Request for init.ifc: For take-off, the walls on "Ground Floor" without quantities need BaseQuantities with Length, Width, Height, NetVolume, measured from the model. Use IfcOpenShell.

First a look at what the model holds.

```python
import ifcopenshell
import ifcopenshell.util.element
import ifcopenshell.util.unit

model = ifcopenshell.open("init.ifc")
print(model.schema)
for unit_type in ("LENGTHUNIT", "AREAUNIT", "VOLUMEUNIT"):
    print(unit_type, ifcopenshell.util.unit.calculate_unit_scale(model, unit_type))
storey = next(s for s in model.by_type("IfcBuildingStorey") if s.Name == "Ground Floor")
walls = [e for e in ifcopenshell.util.element.get_decomposition(storey) if e.is_a("IfcWall")]
for e in sorted(walls, key=lambda e: e.id()):
    print(e.id(), e.is_a(), e.Name, list(ifcopenshell.util.element.get_psets(e, qtos_only=True)), sep=" | ")
```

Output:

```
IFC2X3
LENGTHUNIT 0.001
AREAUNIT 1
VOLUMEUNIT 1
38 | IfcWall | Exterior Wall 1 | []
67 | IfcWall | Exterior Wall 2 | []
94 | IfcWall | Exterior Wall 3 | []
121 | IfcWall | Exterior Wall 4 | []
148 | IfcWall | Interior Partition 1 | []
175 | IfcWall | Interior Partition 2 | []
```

```python
import ifcopenshell
import ifcopenshell.api.pset
import ifcopenshell.geom
import ifcopenshell.util.element
import ifcopenshell.util.shape
import ifcopenshell.util.unit

model = ifcopenshell.open("init.ifc")
unit_scale = ifcopenshell.util.unit.calculate_unit_scale(model)
volume_scale = ifcopenshell.util.unit.calculate_unit_scale(model, "VOLUMEUNIT")
settings = ifcopenshell.geom.settings()

storey = next(s for s in model.by_type("IfcBuildingStorey") if s.Name == "Ground Floor")
walls = [e for e in ifcopenshell.util.element.get_decomposition(storey) if e.is_a("IfcWall")]

for e in sorted(walls, key=lambda e: e.id()):
    if ifcopenshell.util.element.get_psets(e, qtos_only=True, should_inherit=False):
        continue
    # Geometry comes back in metres, in the element's own axes.
    shape = ifcopenshell.geom.create_shape(settings, e)
    values = {
        "Length": ifcopenshell.util.shape.get_x(shape.geometry) / unit_scale,
        "Width": ifcopenshell.util.shape.get_y(shape.geometry) / unit_scale,
        "Height": ifcopenshell.util.shape.get_z(shape.geometry) / unit_scale,
        "NetVolume": ifcopenshell.util.shape.get_volume(shape.geometry) / volume_scale,
    }
    qto = ifcopenshell.api.pset.add_qto(model, product=e, name="BaseQuantities")
    ifcopenshell.api.pset.edit_qto(model, qto=qto, properties=values)
    print(e.id(), {k: round(v, 3) for k, v in values.items()})

model.write("init_rev.ifc")
```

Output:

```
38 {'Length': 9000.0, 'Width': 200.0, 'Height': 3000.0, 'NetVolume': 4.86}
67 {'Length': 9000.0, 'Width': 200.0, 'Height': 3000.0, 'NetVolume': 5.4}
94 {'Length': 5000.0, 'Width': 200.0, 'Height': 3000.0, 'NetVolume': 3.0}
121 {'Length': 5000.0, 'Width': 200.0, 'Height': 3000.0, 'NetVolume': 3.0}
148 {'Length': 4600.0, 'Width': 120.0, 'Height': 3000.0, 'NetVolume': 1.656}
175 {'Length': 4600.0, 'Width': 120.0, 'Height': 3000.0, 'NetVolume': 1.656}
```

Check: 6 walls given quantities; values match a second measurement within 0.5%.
